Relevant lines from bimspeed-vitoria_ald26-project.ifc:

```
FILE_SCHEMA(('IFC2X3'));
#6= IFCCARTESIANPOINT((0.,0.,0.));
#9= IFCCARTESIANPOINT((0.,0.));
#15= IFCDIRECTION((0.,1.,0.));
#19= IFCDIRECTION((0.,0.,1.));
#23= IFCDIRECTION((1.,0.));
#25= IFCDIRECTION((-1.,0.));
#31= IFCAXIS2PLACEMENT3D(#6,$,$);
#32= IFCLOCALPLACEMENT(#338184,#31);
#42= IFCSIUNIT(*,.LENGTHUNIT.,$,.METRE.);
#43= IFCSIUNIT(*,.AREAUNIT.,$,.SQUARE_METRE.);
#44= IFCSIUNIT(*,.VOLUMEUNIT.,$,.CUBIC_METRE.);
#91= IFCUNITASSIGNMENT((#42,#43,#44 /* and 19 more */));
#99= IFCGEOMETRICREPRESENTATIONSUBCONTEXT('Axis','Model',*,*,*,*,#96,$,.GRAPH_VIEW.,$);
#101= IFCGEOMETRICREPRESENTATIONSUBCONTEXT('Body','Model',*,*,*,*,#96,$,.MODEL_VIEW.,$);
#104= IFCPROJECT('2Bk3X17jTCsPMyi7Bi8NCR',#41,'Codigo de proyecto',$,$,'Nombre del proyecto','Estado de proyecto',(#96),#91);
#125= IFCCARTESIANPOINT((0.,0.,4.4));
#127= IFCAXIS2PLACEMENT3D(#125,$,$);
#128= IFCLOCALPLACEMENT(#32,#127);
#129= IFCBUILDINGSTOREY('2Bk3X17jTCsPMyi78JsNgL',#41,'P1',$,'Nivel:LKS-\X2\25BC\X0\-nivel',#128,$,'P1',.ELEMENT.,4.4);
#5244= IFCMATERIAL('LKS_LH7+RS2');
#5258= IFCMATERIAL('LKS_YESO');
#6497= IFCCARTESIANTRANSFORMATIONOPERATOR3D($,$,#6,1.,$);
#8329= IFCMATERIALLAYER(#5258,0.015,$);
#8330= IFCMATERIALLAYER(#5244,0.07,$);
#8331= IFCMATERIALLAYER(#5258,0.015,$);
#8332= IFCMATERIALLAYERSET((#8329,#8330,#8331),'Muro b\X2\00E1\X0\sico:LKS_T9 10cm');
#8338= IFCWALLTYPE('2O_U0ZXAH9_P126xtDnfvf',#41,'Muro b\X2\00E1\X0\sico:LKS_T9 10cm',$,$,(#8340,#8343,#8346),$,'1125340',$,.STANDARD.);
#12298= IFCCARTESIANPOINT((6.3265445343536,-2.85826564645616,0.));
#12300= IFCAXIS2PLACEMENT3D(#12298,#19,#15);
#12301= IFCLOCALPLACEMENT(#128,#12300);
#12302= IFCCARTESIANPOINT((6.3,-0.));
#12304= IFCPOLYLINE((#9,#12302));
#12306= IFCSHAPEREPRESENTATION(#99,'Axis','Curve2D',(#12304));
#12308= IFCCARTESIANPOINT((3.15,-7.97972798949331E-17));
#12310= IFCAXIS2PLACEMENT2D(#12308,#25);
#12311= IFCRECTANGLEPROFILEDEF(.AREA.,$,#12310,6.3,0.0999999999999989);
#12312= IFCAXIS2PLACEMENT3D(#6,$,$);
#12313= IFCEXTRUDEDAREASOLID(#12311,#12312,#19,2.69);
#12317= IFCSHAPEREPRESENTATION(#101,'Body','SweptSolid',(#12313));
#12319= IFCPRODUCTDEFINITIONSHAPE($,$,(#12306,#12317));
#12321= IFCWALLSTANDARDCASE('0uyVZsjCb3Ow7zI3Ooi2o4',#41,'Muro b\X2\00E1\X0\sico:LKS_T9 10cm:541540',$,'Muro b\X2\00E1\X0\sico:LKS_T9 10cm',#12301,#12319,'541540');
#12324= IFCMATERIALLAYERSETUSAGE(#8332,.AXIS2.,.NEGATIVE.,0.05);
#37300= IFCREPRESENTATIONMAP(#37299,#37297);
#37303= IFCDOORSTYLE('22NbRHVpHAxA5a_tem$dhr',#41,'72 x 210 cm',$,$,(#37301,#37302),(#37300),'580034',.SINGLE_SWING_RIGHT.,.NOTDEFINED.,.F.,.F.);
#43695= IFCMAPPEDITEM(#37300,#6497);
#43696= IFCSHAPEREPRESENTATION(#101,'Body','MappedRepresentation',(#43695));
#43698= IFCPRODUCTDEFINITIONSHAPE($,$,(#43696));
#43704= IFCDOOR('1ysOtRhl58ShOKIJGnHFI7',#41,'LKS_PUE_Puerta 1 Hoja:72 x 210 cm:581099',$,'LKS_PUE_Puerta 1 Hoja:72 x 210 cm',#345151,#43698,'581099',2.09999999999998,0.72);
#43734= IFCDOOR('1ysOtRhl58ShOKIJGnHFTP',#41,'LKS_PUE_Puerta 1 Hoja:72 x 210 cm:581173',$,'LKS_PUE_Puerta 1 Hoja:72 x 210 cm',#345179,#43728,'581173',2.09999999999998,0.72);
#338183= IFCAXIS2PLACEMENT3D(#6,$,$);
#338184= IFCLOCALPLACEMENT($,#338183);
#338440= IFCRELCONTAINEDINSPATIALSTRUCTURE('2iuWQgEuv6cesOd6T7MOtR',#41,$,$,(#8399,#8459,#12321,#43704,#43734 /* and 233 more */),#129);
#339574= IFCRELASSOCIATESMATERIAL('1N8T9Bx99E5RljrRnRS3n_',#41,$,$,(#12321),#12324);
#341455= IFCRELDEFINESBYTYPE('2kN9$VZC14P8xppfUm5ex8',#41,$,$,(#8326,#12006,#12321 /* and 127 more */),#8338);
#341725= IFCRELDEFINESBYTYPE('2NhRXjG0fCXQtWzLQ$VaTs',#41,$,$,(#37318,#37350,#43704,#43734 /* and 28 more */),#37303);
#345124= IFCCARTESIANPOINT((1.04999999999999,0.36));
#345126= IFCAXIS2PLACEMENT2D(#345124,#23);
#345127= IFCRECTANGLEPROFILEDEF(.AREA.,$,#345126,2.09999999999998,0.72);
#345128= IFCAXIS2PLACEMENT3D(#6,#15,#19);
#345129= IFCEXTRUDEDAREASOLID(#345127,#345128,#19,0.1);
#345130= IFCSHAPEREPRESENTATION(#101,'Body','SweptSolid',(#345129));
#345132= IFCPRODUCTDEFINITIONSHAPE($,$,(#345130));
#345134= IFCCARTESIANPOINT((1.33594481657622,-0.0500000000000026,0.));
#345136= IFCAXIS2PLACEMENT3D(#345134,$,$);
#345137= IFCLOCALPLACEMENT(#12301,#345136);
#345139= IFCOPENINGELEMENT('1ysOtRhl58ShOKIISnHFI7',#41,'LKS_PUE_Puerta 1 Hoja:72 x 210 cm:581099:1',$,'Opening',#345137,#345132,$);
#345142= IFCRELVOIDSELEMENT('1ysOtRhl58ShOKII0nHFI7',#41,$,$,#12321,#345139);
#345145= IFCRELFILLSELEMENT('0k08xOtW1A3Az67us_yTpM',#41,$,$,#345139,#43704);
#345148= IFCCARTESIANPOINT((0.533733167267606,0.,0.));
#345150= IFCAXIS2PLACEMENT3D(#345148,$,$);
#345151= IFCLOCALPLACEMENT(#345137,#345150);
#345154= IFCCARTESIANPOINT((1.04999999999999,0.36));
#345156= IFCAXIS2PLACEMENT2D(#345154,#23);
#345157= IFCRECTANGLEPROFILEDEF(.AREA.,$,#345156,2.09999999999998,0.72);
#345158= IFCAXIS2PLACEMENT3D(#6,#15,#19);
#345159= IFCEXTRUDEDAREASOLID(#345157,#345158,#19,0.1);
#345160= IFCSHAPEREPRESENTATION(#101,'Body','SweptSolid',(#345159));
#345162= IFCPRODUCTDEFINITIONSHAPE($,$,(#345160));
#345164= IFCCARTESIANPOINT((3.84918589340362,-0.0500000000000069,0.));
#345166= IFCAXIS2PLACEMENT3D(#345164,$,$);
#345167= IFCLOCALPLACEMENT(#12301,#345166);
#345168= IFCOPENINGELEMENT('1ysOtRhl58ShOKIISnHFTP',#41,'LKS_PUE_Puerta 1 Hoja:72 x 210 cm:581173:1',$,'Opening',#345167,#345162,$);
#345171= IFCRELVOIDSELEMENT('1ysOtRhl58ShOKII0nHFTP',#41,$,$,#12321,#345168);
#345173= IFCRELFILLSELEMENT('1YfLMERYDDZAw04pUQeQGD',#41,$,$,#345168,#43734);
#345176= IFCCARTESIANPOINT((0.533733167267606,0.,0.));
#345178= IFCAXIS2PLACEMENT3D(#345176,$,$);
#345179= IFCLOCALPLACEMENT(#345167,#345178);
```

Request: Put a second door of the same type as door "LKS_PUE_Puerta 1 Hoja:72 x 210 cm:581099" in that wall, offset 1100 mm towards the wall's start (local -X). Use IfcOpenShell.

```python
import ifcopenshell
import ifcopenshell.api.feature
import ifcopenshell.api.geometry
import ifcopenshell.api.root
import ifcopenshell.geom
import ifcopenshell.util.element
import ifcopenshell.util.placement
import ifcopenshell.util.shape

model = ifcopenshell.open("bimspeed-vitoria_ald26-project.ifc")
settings = ifcopenshell.geom.settings()


def volume(element):
    """Net volume in cubic metres, openings subtracted."""
    shape = ifcopenshell.geom.create_shape(settings, element)
    return ifcopenshell.util.shape.get_volume(shape.geometry)


def reuse_history(source, copy):
    """copy_class also copies each property set's owner history, people and application; keep the originals."""
    for rel in copy.IsDefinedBy:
        if rel.is_a("IfcRelDefinesByProperties") and (history := rel.RelatingPropertyDefinition.OwnerHistory):
            rel.RelatingPropertyDefinition.OwnerHistory = source.OwnerHistory
            ifcopenshell.util.element.remove_deep2(model, history)


door = model.by_guid("1ysOtRhl58ShOKIJGnHFI7")
opening = door.FillsVoids[0].RelatingOpeningElement
wall = opening.VoidsElements[0].RelatingBuildingElement
before = volume(wall)
shift = ifcopenshell.util.placement.get_local_placement(wall.ObjectPlacement)[:3, 0] * -1.1

# copy_class copies the void relationship, type, container and properties, but no geometry.
new_opening = ifcopenshell.api.root.copy_class(model, product=opening)
new_opening.Representation = ifcopenshell.util.element.copy_deep(
    model, opening.Representation, exclude=["IfcGeometricRepresentationContext", "IfcRepresentationMap"]
)
new_opening.Name = "LKS_PUE_Puerta 1 Hoja:72 x 210 cm"
new_door = ifcopenshell.api.root.copy_class(model, product=door)
new_door.Representation = ifcopenshell.util.element.copy_deep(
    model, door.Representation, exclude=["IfcGeometricRepresentationContext", "IfcRepresentationMap"]
)
new_door.Name = "LKS_PUE_Puerta 1 Hoja:72 x 210 cm"
new_door.Tag = None
reuse_history(door, new_door)
fills = ifcopenshell.api.feature.add_filling(model, opening=new_opening, element=new_door)
fills.OwnerHistory = new_door.OwnerHistory  # required in IFC2X3

for old, new in ((opening, new_opening), (door, new_door)):
    matrix = ifcopenshell.util.placement.get_local_placement(old.ObjectPlacement)
    matrix[:3, 3] += shift
    ifcopenshell.api.geometry.edit_object_placement(model, product=new, matrix=matrix, is_si=False)

after = volume(wall)

print(f"wall volume {before:.3f} -> {after:.3f} m3")

model.write("bimspeed-vitoria_ald26-project_v2.ifc")
```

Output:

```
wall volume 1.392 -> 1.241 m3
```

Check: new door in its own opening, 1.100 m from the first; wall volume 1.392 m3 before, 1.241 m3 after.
